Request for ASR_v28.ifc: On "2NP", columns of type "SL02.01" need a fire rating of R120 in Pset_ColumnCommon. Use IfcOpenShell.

First a look at what the model holds.

```python
import ifcopenshell
import ifcopenshell.util.element

model = ifcopenshell.open("ASR_v28.ifc")
print(model.schema)
storey = next(s for s in model.by_type("IfcBuildingStorey") if s.Name == "2NP")
columns = [e for e in ifcopenshell.util.element.get_decomposition(storey) if e.is_a("IfcColumn")]
seen = {}
for e in columns:
    element_type = ifcopenshell.util.element.get_type(e)
    key = (element_type.Name if element_type != e and element_type else None, ifcopenshell.util.element.get_pset(e, "Pset_ColumnCommon", "FireRating"))
    seen[key] = seen.get(key, 0) + 1
for (name, value), count in sorted(seen.items(), key=str):
    print(count, "x", name, "|", value)
```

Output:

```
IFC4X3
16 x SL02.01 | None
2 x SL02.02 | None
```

```python
import ifcopenshell
import ifcopenshell.api.pset
import ifcopenshell.util.element

model = ifcopenshell.open("ASR_v28.ifc")

storey = next(s for s in model.by_type("IfcBuildingStorey") if s.Name == "2NP")
columns = [e for e in ifcopenshell.util.element.get_decomposition(storey) if e.is_a("IfcColumn")]

count = 0
for e in columns:
    element_type = ifcopenshell.util.element.get_type(e)
    if element_type in (None, e) or element_type.Name != "SL02.01":
        continue
    # add_pset returns the element's existing set when there is one.
    pset = ifcopenshell.api.pset.add_pset(model, product=e, name="Pset_ColumnCommon")
    ifcopenshell.api.pset.edit_pset(model, pset=pset, properties={"FireRating": "R120"})
    count += 1

print(count, "columns updated")

model.write("ASR_v28_updated.ifc")
```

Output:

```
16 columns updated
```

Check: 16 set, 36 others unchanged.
